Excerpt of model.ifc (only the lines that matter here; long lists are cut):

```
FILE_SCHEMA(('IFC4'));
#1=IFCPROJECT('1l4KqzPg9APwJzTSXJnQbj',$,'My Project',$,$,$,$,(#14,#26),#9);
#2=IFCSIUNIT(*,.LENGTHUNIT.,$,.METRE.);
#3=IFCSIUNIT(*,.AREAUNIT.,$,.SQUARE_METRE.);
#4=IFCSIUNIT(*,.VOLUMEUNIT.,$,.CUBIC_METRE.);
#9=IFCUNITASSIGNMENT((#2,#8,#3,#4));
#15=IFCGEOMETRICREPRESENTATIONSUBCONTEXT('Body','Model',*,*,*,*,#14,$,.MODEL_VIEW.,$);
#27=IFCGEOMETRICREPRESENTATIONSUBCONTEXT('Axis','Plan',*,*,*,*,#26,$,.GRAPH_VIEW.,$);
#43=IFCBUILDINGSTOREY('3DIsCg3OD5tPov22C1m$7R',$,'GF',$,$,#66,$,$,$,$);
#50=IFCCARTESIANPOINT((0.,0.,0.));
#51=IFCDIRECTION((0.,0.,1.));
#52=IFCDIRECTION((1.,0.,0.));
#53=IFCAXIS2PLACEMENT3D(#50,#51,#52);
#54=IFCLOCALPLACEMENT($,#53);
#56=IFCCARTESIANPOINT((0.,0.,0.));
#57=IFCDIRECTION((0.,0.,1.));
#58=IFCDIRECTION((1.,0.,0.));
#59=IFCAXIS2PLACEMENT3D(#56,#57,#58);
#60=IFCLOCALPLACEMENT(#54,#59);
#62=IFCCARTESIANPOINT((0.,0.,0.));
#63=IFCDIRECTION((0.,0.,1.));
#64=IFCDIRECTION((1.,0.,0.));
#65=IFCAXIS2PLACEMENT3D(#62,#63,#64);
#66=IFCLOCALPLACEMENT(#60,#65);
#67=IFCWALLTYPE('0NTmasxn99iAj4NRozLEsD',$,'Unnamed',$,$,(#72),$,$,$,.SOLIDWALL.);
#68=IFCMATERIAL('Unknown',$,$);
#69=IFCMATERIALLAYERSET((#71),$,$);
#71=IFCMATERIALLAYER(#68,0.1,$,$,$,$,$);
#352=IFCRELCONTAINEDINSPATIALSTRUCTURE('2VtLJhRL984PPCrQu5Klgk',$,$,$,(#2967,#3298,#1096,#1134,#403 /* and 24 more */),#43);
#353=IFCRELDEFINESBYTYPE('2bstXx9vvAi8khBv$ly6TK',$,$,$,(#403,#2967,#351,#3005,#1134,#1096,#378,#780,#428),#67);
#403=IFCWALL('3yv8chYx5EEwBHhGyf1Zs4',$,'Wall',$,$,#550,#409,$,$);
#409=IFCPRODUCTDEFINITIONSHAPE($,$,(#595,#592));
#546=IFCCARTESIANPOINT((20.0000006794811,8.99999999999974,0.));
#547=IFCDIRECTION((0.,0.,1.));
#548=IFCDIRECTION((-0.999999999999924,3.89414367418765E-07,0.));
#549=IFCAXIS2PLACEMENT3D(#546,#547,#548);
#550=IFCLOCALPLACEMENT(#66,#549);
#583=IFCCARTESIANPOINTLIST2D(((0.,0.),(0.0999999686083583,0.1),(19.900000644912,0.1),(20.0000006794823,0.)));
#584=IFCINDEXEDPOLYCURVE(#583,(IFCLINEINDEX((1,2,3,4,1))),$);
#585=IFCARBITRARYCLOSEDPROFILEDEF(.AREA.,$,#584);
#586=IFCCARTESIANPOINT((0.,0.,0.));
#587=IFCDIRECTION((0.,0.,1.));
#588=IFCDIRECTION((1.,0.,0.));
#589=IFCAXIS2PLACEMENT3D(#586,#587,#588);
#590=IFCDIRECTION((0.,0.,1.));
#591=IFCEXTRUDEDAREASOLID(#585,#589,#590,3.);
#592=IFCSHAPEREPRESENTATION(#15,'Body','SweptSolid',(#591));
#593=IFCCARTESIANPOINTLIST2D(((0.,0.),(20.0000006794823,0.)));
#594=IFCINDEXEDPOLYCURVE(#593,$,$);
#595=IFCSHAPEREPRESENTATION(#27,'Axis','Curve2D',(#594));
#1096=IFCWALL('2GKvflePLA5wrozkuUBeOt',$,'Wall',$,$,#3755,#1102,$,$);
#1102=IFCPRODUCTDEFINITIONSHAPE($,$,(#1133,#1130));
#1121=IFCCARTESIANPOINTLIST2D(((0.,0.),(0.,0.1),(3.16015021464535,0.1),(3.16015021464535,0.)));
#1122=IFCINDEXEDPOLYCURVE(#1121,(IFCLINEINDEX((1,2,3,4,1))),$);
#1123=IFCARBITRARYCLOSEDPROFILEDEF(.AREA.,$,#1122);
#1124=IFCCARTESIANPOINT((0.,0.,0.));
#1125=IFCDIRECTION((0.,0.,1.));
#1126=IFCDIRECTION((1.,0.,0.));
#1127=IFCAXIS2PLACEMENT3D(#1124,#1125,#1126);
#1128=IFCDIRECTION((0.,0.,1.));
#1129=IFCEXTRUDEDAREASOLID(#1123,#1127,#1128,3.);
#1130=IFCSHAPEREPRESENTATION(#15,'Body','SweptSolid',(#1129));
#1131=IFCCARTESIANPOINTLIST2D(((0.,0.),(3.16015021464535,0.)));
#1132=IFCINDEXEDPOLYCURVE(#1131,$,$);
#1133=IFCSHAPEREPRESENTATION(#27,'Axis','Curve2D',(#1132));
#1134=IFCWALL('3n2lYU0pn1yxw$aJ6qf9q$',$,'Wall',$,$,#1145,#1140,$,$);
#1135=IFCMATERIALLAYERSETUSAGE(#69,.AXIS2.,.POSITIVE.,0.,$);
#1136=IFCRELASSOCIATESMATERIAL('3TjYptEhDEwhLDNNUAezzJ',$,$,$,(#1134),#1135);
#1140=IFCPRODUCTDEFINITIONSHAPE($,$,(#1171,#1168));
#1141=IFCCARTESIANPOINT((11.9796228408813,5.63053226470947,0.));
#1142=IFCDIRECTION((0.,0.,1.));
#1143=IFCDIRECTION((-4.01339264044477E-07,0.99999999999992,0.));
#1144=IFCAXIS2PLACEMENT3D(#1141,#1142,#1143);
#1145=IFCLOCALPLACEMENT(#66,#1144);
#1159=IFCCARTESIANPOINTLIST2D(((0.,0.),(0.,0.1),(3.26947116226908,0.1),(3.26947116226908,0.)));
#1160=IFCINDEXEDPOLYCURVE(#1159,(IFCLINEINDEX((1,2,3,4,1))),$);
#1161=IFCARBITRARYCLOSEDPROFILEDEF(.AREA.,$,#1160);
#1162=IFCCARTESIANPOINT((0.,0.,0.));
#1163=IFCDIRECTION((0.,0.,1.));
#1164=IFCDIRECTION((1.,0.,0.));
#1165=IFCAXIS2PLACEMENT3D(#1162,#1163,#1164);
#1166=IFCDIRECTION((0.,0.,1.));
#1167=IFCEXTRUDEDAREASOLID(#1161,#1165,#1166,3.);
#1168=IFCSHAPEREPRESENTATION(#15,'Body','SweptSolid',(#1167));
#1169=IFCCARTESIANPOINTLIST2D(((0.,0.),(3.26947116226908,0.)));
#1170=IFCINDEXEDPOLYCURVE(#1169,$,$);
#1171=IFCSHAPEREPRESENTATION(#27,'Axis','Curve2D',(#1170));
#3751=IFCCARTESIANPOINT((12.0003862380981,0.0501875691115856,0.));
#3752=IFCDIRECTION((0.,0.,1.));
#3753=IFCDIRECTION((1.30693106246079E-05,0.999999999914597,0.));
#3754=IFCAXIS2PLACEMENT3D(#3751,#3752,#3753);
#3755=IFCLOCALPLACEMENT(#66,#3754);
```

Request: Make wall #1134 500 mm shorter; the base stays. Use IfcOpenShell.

```python
import ifcopenshell
import ifcopenshell.geom
import ifcopenshell.util.representation
import ifcopenshell.util.shape

model = ifcopenshell.open("model.ifc")
settings = ifcopenshell.geom.settings()


def volume(element):
    """Net volume in cubic metres, openings subtracted."""
    shape = ifcopenshell.geom.create_shape(settings, element)
    return ifcopenshell.util.shape.get_volume(shape.geometry)


wall = model.by_guid("3n2lYU0pn1yxw$aJ6qf9q$")
before = volume(wall)

body = ifcopenshell.util.representation.get_representation(wall, "Model", "Body")
solid = body.Items[0]
old_height = solid.Depth
solid.Depth -= 0.5
after = volume(wall)

print(f"height {old_height:g} -> {solid.Depth:g}, volume {before:.3f} -> {after:.3f} m3")

model.write("model-out.ifc")
```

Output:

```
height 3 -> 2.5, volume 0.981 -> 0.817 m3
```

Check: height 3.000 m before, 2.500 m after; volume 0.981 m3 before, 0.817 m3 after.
